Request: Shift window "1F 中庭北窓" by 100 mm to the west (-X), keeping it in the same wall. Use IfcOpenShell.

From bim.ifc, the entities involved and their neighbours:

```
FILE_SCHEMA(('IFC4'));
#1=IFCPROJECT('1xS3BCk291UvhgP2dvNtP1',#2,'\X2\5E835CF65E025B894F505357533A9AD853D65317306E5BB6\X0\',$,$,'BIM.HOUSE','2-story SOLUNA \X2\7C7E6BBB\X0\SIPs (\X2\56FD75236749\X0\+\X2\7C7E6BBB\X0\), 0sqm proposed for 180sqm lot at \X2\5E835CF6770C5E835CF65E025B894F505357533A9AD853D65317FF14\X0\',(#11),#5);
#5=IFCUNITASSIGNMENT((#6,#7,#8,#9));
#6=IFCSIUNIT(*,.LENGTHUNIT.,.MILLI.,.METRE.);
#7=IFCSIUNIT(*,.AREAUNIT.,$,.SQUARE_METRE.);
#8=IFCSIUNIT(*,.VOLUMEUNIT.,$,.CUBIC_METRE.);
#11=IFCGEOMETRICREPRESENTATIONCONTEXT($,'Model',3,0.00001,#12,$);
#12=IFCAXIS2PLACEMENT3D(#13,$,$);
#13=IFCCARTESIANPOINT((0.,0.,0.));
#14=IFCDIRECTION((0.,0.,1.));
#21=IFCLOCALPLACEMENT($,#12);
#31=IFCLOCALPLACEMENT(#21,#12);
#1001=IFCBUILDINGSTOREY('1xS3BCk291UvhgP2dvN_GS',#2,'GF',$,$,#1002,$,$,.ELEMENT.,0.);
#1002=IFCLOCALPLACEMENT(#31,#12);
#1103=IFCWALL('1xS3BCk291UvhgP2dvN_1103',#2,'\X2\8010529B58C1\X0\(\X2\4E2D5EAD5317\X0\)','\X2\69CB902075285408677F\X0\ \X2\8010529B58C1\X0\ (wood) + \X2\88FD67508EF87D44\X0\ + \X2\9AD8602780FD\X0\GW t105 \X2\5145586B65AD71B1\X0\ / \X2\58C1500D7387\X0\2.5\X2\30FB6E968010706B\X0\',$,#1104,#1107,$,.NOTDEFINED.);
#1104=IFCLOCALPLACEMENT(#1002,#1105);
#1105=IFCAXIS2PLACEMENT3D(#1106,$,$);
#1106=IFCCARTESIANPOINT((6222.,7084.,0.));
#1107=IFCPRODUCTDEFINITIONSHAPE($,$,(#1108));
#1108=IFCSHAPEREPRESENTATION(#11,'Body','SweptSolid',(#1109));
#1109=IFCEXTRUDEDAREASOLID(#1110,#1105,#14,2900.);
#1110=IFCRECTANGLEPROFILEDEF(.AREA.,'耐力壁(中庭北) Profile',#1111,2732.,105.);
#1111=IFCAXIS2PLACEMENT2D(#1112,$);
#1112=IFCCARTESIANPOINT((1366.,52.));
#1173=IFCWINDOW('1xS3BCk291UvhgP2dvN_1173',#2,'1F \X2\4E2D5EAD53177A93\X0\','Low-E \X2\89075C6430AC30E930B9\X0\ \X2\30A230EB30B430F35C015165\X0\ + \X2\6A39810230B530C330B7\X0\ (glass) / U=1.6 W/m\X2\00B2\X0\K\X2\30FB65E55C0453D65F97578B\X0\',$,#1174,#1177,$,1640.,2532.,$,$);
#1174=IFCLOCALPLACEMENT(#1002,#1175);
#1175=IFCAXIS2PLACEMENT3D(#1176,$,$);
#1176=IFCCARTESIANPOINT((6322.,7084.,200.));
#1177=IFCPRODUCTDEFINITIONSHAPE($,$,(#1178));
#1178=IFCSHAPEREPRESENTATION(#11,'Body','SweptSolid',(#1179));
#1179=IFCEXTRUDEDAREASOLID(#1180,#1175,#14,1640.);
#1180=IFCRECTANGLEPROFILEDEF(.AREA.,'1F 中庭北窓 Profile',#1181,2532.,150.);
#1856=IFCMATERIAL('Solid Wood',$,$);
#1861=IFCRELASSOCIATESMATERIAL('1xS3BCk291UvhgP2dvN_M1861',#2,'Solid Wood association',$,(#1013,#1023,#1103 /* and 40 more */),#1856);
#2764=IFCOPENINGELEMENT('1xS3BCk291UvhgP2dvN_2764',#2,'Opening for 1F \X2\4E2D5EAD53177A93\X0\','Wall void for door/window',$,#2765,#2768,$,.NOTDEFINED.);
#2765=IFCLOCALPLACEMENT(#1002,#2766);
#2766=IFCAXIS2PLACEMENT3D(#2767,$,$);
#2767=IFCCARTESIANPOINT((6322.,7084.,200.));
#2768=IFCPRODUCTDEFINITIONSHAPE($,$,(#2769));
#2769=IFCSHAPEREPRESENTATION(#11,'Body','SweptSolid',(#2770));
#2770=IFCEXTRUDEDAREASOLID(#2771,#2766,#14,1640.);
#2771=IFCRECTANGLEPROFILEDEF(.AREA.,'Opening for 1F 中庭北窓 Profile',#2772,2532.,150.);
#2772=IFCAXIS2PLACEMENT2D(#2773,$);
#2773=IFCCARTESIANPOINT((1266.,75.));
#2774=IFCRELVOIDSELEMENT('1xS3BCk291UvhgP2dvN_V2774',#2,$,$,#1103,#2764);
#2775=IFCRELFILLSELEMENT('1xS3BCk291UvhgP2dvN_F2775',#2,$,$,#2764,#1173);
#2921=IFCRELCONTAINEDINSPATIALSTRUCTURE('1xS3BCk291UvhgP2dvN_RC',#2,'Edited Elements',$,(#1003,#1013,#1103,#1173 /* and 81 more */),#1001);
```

```python
import ifcopenshell
import ifcopenshell.api.geometry
import ifcopenshell.util.placement
import ifcopenshell.util.unit

model = ifcopenshell.open("bim.ifc")
unit_scale = ifcopenshell.util.unit.calculate_unit_scale(model)

window = model.by_guid("1xS3BCk291UvhgP2dvN_1173")
opening = window.FillsVoids[0].RelatingOpeningElement
wall = opening.VoidsElements[0].RelatingBuildingElement

wall_matrix = ifcopenshell.util.placement.get_local_placement(wall.ObjectPlacement)
shift = wall_matrix[:3, 0] * -0.1 / unit_scale
before = ifcopenshell.util.placement.get_local_placement(window.ObjectPlacement)[:3, 3].copy()

# The window is not placed relative to its opening, so move both.
for product in (opening, window):
    matrix = ifcopenshell.util.placement.get_local_placement(product.ObjectPlacement)
    matrix[:3, 3] += shift
    ifcopenshell.api.geometry.edit_object_placement(model, product=product, matrix=matrix, is_si=False)

after = ifcopenshell.util.placement.get_local_placement(window.ObjectPlacement)[:3, 3]
print("window moved by", (after - before).round(3) + 0.0)

model.write("bim_rev.ifc")
```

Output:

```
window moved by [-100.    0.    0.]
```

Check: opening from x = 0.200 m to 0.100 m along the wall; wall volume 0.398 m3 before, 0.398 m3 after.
